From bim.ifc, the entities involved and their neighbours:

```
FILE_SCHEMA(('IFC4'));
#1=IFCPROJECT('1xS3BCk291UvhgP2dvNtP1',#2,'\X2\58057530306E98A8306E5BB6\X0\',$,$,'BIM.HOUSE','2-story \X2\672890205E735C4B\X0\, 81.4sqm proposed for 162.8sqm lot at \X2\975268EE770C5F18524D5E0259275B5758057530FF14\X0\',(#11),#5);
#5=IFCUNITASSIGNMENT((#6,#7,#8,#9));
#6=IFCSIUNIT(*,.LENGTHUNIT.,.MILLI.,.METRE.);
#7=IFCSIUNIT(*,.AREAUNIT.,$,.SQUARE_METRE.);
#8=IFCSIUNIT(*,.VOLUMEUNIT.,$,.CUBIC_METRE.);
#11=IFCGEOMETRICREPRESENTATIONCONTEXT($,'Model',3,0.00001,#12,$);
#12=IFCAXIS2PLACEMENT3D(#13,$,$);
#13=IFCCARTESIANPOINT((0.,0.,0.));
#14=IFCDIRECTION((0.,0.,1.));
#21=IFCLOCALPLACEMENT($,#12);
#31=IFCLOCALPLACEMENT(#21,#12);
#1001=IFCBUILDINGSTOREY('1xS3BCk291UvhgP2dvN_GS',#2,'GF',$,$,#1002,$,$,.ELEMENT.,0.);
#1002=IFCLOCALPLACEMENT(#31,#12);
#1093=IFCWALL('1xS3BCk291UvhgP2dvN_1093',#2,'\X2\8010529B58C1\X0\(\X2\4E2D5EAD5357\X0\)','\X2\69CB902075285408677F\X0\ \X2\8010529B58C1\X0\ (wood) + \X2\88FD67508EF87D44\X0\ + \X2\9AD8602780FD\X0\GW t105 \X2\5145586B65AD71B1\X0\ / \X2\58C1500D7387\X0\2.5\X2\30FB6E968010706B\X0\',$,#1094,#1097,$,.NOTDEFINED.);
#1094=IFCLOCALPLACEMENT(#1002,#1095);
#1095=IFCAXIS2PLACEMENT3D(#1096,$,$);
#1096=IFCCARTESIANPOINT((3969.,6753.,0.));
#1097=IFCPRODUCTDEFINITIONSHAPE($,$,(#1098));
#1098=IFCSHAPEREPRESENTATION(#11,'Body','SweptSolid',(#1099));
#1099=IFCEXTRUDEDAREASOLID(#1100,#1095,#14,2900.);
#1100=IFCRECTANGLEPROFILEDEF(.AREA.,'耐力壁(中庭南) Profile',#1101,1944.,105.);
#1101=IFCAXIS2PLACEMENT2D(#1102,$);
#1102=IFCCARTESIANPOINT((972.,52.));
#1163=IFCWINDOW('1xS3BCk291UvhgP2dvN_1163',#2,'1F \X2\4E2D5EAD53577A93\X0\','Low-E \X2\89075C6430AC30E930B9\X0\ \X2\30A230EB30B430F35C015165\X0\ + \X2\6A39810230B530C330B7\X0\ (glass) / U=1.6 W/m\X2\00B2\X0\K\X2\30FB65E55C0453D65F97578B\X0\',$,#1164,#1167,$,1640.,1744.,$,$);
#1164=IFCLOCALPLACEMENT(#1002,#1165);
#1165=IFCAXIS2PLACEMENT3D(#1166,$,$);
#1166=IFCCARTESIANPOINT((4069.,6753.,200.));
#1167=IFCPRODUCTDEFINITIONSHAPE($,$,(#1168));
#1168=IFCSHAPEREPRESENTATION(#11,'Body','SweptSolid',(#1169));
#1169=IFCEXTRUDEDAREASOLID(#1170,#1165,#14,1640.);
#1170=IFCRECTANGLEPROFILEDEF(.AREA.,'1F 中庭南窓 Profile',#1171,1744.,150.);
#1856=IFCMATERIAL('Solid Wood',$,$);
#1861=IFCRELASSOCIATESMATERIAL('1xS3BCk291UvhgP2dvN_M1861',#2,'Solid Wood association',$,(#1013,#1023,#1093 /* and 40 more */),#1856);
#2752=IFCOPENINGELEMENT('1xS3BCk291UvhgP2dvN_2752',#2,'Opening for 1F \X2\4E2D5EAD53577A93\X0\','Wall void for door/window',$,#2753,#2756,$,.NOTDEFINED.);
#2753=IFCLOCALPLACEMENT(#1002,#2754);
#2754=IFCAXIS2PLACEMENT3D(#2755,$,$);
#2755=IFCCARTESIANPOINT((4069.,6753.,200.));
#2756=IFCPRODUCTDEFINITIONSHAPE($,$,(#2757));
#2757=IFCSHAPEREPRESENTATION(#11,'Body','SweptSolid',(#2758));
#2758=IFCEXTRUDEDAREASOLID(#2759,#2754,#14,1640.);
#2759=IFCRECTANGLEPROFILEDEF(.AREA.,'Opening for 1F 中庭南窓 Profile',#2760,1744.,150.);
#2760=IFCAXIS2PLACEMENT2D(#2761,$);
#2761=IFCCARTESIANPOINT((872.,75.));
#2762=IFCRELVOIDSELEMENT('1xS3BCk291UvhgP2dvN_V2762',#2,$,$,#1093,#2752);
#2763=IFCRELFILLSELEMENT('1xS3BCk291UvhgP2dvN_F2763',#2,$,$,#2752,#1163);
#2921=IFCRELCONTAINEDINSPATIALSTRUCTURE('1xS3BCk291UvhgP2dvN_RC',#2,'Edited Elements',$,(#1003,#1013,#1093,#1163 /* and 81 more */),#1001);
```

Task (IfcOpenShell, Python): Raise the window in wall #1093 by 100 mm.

```python
import numpy as np
import ifcopenshell
import ifcopenshell.api.geometry
import ifcopenshell.util.placement
import ifcopenshell.util.unit

model = ifcopenshell.open("bim.ifc")
unit_scale = ifcopenshell.util.unit.calculate_unit_scale(model)

window = model.by_guid("1xS3BCk291UvhgP2dvN_1163")
opening = window.FillsVoids[0].RelatingOpeningElement
dz = 0.1 / unit_scale

shift = np.array([0.0, 0.0, dz])
# The window is not placed relative to its opening, so move both.
for product in (opening, window):
    matrix = ifcopenshell.util.placement.get_local_placement(product.ObjectPlacement)
    matrix[:3, 3] += shift
    ifcopenshell.api.geometry.edit_object_placement(model, product=product, matrix=matrix, is_si=False)

print(f"moved by {dz * unit_scale:+.3f} m")

model.write("bim-out.ifc")
```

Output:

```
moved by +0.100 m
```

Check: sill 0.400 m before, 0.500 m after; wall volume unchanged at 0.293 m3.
